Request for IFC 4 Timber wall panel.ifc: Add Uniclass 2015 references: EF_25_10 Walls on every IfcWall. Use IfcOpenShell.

First a look at what the model holds.

```python
import ifcopenshell

model = ifcopenshell.open("IFC 4 Timber wall panel.ifc")
print(model.schema)
print("classifications:", [c.Name for c in model.by_type("IfcClassification")])
for ifc_class in ("IfcDoor", "IfcRoof", "IfcStair", "IfcWall", "IfcWindow"):
    print(ifc_class, len(model.by_type(ifc_class)))
```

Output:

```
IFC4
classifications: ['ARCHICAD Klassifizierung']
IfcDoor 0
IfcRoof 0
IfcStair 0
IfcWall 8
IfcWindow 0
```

```python
import ifcopenshell
import ifcopenshell.api.classification

model = ifcopenshell.open("IFC 4 Timber wall panel.ifc")

system = ifcopenshell.api.classification.add_classification(model, classification="Uniclass 2015")

codes = {
    "IfcWall": ("EF_25_10", "Walls"),
}
for ifc_class, (code, name) in codes.items():
    products = model.by_type(ifc_class)
    ifcopenshell.api.classification.add_reference(
        model, products=products, classification=system, identification=code, name=name
    )
    print(code, len(products))

model.write("IFC 4 Timber wall panel_rev.ifc")
```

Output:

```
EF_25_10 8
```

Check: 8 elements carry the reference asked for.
